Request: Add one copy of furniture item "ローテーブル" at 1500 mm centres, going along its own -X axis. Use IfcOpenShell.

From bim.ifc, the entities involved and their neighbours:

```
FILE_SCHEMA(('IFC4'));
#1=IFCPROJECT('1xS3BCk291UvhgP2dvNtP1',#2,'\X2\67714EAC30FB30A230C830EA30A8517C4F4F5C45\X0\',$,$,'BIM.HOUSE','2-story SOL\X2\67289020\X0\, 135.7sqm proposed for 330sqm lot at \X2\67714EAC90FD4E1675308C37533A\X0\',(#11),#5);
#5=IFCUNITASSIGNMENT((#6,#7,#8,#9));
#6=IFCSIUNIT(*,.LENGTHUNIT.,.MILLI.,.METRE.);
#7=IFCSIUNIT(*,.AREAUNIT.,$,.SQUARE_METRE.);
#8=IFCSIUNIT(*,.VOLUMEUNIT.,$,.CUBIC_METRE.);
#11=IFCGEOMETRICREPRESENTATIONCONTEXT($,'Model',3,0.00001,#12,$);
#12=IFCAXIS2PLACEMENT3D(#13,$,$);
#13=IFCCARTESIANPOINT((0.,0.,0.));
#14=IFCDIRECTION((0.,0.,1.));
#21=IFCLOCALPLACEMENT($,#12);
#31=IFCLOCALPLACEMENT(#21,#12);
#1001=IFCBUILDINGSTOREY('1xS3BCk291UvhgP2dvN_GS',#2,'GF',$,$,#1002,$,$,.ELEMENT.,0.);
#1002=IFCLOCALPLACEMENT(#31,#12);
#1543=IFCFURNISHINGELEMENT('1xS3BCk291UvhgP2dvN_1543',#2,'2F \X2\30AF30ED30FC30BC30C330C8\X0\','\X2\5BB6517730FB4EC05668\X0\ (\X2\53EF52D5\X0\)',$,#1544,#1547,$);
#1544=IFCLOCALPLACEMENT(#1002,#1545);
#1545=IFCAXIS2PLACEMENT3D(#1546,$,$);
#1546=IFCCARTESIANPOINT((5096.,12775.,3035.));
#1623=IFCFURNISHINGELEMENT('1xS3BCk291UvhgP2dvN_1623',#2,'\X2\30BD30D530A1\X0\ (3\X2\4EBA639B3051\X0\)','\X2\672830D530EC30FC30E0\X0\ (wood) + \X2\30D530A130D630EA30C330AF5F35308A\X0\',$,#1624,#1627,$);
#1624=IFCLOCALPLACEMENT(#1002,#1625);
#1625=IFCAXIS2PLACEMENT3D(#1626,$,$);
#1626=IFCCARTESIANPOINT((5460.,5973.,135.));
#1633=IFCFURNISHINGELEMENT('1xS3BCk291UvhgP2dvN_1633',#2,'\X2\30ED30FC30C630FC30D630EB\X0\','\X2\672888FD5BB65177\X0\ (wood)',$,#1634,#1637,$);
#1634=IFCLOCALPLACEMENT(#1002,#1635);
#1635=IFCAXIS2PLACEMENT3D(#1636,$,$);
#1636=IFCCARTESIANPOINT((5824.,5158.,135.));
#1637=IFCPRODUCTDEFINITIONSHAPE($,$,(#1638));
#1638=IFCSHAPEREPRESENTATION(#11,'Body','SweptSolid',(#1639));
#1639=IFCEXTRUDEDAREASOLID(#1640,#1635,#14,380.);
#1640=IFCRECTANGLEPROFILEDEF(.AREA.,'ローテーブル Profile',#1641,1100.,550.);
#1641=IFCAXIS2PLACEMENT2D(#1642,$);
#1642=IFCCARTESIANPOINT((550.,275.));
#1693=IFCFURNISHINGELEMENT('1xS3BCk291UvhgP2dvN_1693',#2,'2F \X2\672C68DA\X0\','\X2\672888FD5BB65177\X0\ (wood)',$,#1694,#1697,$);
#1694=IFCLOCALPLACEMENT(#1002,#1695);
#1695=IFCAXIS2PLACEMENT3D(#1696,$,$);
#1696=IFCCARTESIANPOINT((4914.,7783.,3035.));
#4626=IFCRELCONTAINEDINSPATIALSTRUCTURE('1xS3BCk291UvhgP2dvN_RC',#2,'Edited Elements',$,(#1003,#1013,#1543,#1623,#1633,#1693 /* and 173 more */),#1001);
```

```python
import ifcopenshell
import ifcopenshell.api.geometry
import ifcopenshell.api.root
import ifcopenshell.util.element
import ifcopenshell.util.placement

model = ifcopenshell.open("bim.ifc")


def reuse_history(source, copy):
    """copy_class also copies each property set's owner history, people and application; keep the originals."""
    for rel in copy.IsDefinedBy:
        if rel.is_a("IfcRelDefinesByProperties") and (history := rel.RelatingPropertyDefinition.OwnerHistory):
            rel.RelatingPropertyDefinition.OwnerHistory = source.OwnerHistory
            ifcopenshell.util.element.remove_deep2(model, history)


source = model.by_id(1633)
base = ifcopenshell.util.placement.get_local_placement(source.ObjectPlacement)
step = -base[:3, 0] * 1500.0

for i in range(1, 2):
    copy = ifcopenshell.api.root.copy_class(model, product=source)
    copy.Representation = ifcopenshell.util.element.copy_deep(
        model, source.Representation, exclude=["IfcGeometricRepresentationContext", "IfcRepresentationMap"]
    )
    reuse_history(source, copy)
    matrix = base.copy()
    matrix[:3, 3] += i * step
    print("added at", matrix[:3, 3].round(3) + 0.0)
    ifcopenshell.api.geometry.edit_object_placement(model, product=copy, matrix=matrix, is_si=False)

model.write("bim-out.ifc")
```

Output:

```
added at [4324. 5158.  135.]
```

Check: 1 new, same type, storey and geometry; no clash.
